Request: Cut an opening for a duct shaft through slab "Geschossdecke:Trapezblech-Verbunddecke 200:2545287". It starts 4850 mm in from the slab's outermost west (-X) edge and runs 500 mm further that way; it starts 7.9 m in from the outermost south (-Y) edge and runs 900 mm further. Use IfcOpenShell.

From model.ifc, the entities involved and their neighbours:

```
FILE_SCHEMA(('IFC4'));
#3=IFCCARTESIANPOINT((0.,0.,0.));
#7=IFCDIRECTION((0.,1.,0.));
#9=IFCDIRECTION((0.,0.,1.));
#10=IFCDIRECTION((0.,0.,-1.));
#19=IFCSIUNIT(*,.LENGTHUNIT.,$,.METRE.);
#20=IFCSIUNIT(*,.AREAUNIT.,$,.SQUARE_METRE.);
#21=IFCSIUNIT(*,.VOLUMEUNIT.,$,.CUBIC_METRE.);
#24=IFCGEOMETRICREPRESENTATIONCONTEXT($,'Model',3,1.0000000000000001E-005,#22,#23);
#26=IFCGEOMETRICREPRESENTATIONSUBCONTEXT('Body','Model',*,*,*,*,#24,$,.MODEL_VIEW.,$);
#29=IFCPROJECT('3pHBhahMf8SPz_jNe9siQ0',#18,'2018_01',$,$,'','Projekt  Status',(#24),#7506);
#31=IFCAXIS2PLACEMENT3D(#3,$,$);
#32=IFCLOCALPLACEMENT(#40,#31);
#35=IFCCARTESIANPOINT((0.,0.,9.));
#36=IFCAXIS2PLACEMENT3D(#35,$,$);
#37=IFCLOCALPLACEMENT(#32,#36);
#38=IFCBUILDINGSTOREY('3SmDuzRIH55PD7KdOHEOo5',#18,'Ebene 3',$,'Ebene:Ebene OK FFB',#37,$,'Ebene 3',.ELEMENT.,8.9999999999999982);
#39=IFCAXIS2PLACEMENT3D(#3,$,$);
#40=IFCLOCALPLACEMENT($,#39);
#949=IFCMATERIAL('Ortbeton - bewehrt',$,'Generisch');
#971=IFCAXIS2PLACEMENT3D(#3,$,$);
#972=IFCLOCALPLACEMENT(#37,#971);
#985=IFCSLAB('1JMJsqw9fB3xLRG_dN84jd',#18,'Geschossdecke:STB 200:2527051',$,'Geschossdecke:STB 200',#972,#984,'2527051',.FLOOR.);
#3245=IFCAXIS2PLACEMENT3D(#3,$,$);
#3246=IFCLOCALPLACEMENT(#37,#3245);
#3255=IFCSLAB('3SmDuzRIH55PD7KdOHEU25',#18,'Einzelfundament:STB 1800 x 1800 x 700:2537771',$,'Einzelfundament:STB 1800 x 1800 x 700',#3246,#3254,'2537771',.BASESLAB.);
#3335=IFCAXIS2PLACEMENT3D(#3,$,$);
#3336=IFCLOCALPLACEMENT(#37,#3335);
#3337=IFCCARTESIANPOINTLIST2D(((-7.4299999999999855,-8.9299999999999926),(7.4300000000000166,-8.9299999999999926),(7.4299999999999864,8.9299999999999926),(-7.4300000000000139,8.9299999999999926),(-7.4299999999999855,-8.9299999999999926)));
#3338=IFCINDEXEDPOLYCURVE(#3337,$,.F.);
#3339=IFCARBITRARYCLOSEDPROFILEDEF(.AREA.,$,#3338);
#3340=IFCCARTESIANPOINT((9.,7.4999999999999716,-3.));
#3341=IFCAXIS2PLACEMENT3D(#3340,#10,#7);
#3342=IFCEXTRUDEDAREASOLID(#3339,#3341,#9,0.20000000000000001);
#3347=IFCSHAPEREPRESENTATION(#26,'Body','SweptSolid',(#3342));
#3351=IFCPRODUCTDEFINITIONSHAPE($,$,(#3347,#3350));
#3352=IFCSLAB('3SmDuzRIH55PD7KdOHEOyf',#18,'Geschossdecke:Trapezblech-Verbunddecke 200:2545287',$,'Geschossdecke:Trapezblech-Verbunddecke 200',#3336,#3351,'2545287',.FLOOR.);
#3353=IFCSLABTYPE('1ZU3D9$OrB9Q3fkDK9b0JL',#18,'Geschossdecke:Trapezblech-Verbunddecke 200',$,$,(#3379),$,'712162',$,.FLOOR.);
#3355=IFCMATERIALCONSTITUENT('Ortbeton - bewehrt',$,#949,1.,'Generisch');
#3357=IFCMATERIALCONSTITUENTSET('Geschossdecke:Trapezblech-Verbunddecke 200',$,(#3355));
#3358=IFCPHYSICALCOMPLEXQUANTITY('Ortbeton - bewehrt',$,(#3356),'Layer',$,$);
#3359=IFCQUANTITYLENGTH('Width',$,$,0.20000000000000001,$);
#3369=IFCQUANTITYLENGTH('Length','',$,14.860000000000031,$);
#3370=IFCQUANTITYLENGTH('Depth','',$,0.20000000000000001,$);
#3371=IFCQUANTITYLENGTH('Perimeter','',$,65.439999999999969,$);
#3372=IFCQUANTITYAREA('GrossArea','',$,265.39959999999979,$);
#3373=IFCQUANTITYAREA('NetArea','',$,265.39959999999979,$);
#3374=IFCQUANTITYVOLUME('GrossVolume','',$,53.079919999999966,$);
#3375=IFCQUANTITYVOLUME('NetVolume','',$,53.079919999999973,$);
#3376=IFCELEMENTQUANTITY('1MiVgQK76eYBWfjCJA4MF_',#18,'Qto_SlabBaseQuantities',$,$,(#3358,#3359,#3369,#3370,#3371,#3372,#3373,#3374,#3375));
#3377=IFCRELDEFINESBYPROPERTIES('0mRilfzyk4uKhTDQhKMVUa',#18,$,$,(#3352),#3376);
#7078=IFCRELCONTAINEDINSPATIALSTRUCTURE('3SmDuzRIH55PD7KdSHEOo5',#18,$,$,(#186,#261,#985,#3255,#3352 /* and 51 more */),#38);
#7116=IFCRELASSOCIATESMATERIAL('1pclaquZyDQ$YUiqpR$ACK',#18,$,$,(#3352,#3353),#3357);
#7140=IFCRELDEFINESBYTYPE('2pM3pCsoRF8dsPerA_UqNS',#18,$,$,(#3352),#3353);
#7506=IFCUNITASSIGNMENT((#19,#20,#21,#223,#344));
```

```python
import numpy as np
import ifcopenshell
import ifcopenshell.api.feature
import ifcopenshell.api.geometry
import ifcopenshell.api.pset
import ifcopenshell.api.root
import ifcopenshell.geom
import ifcopenshell.util.element
import ifcopenshell.util.placement
import ifcopenshell.util.representation
import ifcopenshell.util.shape
import ifcopenshell.util.unit

model = ifcopenshell.open("model.ifc")
unit_scale = ifcopenshell.util.unit.calculate_unit_scale(model)
area_scale = ifcopenshell.util.unit.calculate_unit_scale(model, "AREAUNIT")
volume_scale = ifcopenshell.util.unit.calculate_unit_scale(model, "VOLUMEUNIT")
settings = ifcopenshell.geom.settings()


def volume(element):
    """Net volume in cubic metres, openings subtracted."""
    shape = ifcopenshell.geom.create_shape(settings, element)
    return ifcopenshell.util.shape.get_volume(shape.geometry)


slab = model.by_guid("3SmDuzRIH55PD7KdOHEOyf")
before = volume(slab)

# Extent in the slab's own axes, in metres. The edges named are its -X and -Y sides.
slab_shape = ifcopenshell.geom.create_shape(settings, slab)
vertices = ifcopenshell.util.shape.get_vertices(slab_shape.geometry)
x_min, y_min, bottom = vertices.min(axis=0)
top = vertices[:, 2].max()

opening = ifcopenshell.api.root.create_entity(model, ifc_class="IfcOpeningElement", name="Duct shaft opening", predefined_type="OPENING")
context = ifcopenshell.util.representation.get_context(model, "Model", "Body", "MODEL_VIEW")
width, depth = 0.5, 0.9
outline = [(0.0, 0.0), (width, 0.0), (width, depth), (0.0, depth), (0.0, 0.0)]
# Overshoot both faces by 50 mm so the cut is clean.
shape = ifcopenshell.api.geometry.add_slab_representation(
    model, context=context, depth=top - bottom + 0.1, polyline=outline
)
ifcopenshell.api.geometry.assign_representation(model, product=opening, representation=shape)

matrix = ifcopenshell.util.placement.get_local_placement(slab.ObjectPlacement)
matrix[:, 3] = matrix @ np.append(np.array([x_min + 4.85, y_min + 7.9, bottom - 0.05]) / unit_scale, 1.0)
ifcopenshell.api.geometry.edit_object_placement(model, product=opening, matrix=matrix, is_si=False)
ifcopenshell.api.feature.add_feature(model, feature=opening, element=slab)

after = volume(slab)

# Update the slab's stored quantities.
qto = model.by_id(ifcopenshell.util.element.get_pset(slab, "Qto_SlabBaseQuantities", should_inherit=False)["id"])
ifcopenshell.api.pset.edit_qto(model, qto=qto, properties={
    "NetArea": after / (top - bottom) / area_scale,
    "NetVolume": after / volume_scale,
})

print(f"slab volume {before:.3f} -> {after:.3f} m3")

model.write("model_updated.ifc")
```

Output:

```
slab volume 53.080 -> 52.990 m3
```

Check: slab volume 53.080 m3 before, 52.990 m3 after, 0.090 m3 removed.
